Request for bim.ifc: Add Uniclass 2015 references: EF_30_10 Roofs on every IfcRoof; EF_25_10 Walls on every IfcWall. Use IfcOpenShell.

First a look at what the model holds.

```python
import ifcopenshell

model = ifcopenshell.open("bim.ifc")
print(model.schema)
print("classifications:", [c.Name for c in model.by_type("IfcClassification")])
for ifc_class in ("IfcDoor", "IfcRoof", "IfcStair", "IfcWall", "IfcWindow"):
    print(ifc_class, len(model.by_type(ifc_class)))
```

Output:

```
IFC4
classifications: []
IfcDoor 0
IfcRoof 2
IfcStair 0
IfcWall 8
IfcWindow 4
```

```python
import ifcopenshell
import ifcopenshell.api.classification

model = ifcopenshell.open("bim.ifc")

system = ifcopenshell.api.classification.add_classification(model, classification="Uniclass 2015")

codes = {
    "IfcRoof": ("EF_30_10", "Roofs"),
    "IfcWall": ("EF_25_10", "Walls"),
}
for ifc_class, (code, name) in codes.items():
    products = model.by_type(ifc_class)
    ifcopenshell.api.classification.add_reference(
        model, products=products, classification=system, identification=code, name=name
    )
    print(code, len(products))

model.write("bim_rev.ifc")
```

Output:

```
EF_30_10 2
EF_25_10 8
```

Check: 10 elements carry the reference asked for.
